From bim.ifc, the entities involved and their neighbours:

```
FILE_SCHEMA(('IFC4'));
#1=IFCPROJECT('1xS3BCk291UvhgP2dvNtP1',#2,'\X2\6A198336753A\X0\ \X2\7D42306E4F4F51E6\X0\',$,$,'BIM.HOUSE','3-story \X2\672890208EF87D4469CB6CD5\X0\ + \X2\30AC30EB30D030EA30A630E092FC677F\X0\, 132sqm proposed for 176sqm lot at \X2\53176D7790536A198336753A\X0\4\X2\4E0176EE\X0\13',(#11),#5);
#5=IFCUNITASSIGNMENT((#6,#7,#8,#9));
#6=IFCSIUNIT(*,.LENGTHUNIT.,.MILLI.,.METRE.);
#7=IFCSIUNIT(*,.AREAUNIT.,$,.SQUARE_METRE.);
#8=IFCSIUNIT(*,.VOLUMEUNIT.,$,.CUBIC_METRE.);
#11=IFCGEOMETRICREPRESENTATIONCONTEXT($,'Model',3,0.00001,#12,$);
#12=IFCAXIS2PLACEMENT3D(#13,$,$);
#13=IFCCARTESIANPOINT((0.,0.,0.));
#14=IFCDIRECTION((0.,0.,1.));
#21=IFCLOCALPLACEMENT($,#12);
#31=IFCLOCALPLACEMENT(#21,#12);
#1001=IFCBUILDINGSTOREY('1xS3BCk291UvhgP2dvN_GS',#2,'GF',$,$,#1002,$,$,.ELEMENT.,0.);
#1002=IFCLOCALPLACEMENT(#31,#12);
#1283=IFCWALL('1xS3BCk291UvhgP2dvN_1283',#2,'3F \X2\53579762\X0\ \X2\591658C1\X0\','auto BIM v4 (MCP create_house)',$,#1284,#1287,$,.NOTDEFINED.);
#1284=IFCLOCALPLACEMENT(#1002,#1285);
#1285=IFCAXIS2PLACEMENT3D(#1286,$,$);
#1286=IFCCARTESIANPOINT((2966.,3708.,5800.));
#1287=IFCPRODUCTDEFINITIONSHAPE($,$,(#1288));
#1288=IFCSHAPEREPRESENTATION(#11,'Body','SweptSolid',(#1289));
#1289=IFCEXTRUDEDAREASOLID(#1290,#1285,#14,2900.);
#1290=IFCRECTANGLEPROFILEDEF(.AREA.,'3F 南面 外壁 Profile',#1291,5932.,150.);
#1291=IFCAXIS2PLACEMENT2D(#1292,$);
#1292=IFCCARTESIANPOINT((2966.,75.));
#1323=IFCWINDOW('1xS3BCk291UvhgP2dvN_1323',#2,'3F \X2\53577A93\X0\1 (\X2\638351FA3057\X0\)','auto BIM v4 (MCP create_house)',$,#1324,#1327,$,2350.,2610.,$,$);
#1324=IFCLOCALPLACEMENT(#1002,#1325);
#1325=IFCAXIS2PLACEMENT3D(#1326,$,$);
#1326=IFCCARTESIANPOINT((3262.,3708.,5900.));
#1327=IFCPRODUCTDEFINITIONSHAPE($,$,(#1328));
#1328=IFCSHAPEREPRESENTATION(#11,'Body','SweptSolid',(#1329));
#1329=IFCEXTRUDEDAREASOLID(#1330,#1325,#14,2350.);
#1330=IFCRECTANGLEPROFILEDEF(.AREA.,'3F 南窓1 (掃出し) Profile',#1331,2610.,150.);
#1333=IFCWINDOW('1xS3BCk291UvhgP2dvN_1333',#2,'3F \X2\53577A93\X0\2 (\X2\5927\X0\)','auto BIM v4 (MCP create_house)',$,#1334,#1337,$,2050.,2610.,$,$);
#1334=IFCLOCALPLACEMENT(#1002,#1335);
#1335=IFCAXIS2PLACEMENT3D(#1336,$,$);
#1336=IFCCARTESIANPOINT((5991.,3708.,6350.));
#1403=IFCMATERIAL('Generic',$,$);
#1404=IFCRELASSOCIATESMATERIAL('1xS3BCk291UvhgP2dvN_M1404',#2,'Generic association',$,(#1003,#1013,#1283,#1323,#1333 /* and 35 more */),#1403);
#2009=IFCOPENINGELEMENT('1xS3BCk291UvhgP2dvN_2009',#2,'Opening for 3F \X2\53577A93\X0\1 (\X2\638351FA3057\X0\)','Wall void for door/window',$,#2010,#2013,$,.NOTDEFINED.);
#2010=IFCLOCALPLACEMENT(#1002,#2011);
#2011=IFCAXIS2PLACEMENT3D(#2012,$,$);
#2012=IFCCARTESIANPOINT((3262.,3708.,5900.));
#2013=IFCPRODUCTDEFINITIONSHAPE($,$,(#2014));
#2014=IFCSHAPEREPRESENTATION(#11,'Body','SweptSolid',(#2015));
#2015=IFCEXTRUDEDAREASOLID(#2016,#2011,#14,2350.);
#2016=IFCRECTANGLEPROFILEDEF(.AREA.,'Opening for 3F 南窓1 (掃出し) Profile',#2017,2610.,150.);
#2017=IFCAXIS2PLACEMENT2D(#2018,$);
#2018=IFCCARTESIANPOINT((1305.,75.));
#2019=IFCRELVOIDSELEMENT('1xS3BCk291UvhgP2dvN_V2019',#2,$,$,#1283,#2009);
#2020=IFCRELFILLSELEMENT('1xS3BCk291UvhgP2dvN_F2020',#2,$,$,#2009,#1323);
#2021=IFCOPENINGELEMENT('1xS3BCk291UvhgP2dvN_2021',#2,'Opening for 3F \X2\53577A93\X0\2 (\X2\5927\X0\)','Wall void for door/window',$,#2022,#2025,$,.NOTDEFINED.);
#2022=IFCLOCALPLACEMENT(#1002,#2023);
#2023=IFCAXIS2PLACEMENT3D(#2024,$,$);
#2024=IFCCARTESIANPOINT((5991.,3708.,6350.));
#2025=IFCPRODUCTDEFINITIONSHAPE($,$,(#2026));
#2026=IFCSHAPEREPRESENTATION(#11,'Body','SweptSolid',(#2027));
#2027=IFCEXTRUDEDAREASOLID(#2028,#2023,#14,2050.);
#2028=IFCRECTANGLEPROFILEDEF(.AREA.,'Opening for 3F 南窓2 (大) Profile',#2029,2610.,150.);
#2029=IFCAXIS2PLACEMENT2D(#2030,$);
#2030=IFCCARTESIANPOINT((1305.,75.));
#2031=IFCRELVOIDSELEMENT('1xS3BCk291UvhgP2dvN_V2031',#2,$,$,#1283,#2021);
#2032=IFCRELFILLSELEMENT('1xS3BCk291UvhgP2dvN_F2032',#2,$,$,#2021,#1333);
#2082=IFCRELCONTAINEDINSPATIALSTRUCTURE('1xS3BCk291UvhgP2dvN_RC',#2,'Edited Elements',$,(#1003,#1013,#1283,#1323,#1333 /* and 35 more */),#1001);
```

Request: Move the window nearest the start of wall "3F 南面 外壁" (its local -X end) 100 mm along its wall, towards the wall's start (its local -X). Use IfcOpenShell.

```python
import ifcopenshell
import ifcopenshell.api.geometry
import ifcopenshell.util.placement
import ifcopenshell.util.unit

model = ifcopenshell.open("bim.ifc")
unit_scale = ifcopenshell.util.unit.calculate_unit_scale(model)

window = model.by_guid("1xS3BCk291UvhgP2dvN_1323")
opening = window.FillsVoids[0].RelatingOpeningElement
wall = opening.VoidsElements[0].RelatingBuildingElement

wall_matrix = ifcopenshell.util.placement.get_local_placement(wall.ObjectPlacement)
shift = wall_matrix[:3, 0] * -0.1 / unit_scale
before = ifcopenshell.util.placement.get_local_placement(window.ObjectPlacement)[:3, 3].copy()

# The window is not placed relative to its opening, so move both.
for product in (opening, window):
    matrix = ifcopenshell.util.placement.get_local_placement(product.ObjectPlacement)
    matrix[:3, 3] += shift
    ifcopenshell.api.geometry.edit_object_placement(model, product=product, matrix=matrix, is_si=False)

after = ifcopenshell.util.placement.get_local_placement(window.ObjectPlacement)[:3, 3]
print("window moved by", (after - before).round(3) + 0.0)

model.write("bim-out.ifc")
```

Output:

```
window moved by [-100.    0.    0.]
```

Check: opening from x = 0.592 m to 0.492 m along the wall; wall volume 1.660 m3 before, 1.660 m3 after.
